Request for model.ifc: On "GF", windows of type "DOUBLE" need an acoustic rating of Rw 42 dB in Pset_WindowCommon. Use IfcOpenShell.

First a look at what the model holds.

```python
import ifcopenshell
import ifcopenshell.util.element

model = ifcopenshell.open("model.ifc")
print(model.schema)
storey = next(s for s in model.by_type("IfcBuildingStorey") if s.Name == "GF")
windows = [e for e in ifcopenshell.util.element.get_decomposition(storey) if e.is_a("IfcWindow")]
seen = {}
for e in windows:
    element_type = ifcopenshell.util.element.get_type(e)
    key = (element_type.Name if element_type != e and element_type else None, ifcopenshell.util.element.get_pset(e, "Pset_WindowCommon", "AcousticRating"))
    seen[key] = seen.get(key, 0) + 1
for (name, value), count in sorted(seen.items(), key=str):
    print(count, "x", name, "|", value)
```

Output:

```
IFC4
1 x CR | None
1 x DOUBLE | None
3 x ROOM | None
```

```python
import ifcopenshell
import ifcopenshell.api.pset
import ifcopenshell.util.element

model = ifcopenshell.open("model.ifc")

storey = next(s for s in model.by_type("IfcBuildingStorey") if s.Name == "GF")
windows = [e for e in ifcopenshell.util.element.get_decomposition(storey) if e.is_a("IfcWindow")]

count = 0
for e in windows:
    element_type = ifcopenshell.util.element.get_type(e)
    if element_type in (None, e) or element_type.Name != "DOUBLE":
        continue
    # add_pset returns the element's existing set when there is one.
    pset = ifcopenshell.api.pset.add_pset(model, product=e, name="Pset_WindowCommon")
    ifcopenshell.api.pset.edit_pset(model, pset=pset, properties={"AcousticRating": "Rw 42 dB"})
    count += 1

print(count, "windows updated")

model.write("model-out.ifc")
```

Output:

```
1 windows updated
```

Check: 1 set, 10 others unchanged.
